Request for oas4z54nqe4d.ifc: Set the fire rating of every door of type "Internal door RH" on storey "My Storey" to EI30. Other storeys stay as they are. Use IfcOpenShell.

First a look at what the model holds.

```python
import ifcopenshell
import ifcopenshell.util.element

model = ifcopenshell.open("oas4z54nqe4d.ifc")
print(model.schema)
storey = next(s for s in model.by_type("IfcBuildingStorey") if s.Name == "My Storey")
doors = [e for e in ifcopenshell.util.element.get_decomposition(storey) if e.is_a("IfcDoor")]
seen = {}
for e in doors:
    element_type = ifcopenshell.util.element.get_type(e)
    key = (element_type.Name if element_type != e and element_type else None, ifcopenshell.util.element.get_pset(e, "Pset_DoorCommon", "FireRating"))
    seen[key] = seen.get(key, 0) + 1
for (name, value), count in sorted(seen.items(), key=str):
    print(count, "x", name, "|", value)
```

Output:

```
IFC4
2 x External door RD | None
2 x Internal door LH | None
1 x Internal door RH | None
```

```python
import ifcopenshell
import ifcopenshell.api.pset
import ifcopenshell.util.element

model = ifcopenshell.open("oas4z54nqe4d.ifc")

storey = next(s for s in model.by_type("IfcBuildingStorey") if s.Name == "My Storey")
doors = [e for e in ifcopenshell.util.element.get_decomposition(storey) if e.is_a("IfcDoor")]

count = 0
for e in doors:
    element_type = ifcopenshell.util.element.get_type(e)
    if element_type in (None, e) or element_type.Name != "Internal door RH":
        continue
    # add_pset returns the element's existing set when there is one.
    pset = ifcopenshell.api.pset.add_pset(model, product=e, name="Pset_DoorCommon")
    ifcopenshell.api.pset.edit_pset(model, pset=pset, properties={"FireRating": "EI30"})
    count += 1

print(count, "doors updated")

model.write("oas4z54nqe4d_v2.ifc")
```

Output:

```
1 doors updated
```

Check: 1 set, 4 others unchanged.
